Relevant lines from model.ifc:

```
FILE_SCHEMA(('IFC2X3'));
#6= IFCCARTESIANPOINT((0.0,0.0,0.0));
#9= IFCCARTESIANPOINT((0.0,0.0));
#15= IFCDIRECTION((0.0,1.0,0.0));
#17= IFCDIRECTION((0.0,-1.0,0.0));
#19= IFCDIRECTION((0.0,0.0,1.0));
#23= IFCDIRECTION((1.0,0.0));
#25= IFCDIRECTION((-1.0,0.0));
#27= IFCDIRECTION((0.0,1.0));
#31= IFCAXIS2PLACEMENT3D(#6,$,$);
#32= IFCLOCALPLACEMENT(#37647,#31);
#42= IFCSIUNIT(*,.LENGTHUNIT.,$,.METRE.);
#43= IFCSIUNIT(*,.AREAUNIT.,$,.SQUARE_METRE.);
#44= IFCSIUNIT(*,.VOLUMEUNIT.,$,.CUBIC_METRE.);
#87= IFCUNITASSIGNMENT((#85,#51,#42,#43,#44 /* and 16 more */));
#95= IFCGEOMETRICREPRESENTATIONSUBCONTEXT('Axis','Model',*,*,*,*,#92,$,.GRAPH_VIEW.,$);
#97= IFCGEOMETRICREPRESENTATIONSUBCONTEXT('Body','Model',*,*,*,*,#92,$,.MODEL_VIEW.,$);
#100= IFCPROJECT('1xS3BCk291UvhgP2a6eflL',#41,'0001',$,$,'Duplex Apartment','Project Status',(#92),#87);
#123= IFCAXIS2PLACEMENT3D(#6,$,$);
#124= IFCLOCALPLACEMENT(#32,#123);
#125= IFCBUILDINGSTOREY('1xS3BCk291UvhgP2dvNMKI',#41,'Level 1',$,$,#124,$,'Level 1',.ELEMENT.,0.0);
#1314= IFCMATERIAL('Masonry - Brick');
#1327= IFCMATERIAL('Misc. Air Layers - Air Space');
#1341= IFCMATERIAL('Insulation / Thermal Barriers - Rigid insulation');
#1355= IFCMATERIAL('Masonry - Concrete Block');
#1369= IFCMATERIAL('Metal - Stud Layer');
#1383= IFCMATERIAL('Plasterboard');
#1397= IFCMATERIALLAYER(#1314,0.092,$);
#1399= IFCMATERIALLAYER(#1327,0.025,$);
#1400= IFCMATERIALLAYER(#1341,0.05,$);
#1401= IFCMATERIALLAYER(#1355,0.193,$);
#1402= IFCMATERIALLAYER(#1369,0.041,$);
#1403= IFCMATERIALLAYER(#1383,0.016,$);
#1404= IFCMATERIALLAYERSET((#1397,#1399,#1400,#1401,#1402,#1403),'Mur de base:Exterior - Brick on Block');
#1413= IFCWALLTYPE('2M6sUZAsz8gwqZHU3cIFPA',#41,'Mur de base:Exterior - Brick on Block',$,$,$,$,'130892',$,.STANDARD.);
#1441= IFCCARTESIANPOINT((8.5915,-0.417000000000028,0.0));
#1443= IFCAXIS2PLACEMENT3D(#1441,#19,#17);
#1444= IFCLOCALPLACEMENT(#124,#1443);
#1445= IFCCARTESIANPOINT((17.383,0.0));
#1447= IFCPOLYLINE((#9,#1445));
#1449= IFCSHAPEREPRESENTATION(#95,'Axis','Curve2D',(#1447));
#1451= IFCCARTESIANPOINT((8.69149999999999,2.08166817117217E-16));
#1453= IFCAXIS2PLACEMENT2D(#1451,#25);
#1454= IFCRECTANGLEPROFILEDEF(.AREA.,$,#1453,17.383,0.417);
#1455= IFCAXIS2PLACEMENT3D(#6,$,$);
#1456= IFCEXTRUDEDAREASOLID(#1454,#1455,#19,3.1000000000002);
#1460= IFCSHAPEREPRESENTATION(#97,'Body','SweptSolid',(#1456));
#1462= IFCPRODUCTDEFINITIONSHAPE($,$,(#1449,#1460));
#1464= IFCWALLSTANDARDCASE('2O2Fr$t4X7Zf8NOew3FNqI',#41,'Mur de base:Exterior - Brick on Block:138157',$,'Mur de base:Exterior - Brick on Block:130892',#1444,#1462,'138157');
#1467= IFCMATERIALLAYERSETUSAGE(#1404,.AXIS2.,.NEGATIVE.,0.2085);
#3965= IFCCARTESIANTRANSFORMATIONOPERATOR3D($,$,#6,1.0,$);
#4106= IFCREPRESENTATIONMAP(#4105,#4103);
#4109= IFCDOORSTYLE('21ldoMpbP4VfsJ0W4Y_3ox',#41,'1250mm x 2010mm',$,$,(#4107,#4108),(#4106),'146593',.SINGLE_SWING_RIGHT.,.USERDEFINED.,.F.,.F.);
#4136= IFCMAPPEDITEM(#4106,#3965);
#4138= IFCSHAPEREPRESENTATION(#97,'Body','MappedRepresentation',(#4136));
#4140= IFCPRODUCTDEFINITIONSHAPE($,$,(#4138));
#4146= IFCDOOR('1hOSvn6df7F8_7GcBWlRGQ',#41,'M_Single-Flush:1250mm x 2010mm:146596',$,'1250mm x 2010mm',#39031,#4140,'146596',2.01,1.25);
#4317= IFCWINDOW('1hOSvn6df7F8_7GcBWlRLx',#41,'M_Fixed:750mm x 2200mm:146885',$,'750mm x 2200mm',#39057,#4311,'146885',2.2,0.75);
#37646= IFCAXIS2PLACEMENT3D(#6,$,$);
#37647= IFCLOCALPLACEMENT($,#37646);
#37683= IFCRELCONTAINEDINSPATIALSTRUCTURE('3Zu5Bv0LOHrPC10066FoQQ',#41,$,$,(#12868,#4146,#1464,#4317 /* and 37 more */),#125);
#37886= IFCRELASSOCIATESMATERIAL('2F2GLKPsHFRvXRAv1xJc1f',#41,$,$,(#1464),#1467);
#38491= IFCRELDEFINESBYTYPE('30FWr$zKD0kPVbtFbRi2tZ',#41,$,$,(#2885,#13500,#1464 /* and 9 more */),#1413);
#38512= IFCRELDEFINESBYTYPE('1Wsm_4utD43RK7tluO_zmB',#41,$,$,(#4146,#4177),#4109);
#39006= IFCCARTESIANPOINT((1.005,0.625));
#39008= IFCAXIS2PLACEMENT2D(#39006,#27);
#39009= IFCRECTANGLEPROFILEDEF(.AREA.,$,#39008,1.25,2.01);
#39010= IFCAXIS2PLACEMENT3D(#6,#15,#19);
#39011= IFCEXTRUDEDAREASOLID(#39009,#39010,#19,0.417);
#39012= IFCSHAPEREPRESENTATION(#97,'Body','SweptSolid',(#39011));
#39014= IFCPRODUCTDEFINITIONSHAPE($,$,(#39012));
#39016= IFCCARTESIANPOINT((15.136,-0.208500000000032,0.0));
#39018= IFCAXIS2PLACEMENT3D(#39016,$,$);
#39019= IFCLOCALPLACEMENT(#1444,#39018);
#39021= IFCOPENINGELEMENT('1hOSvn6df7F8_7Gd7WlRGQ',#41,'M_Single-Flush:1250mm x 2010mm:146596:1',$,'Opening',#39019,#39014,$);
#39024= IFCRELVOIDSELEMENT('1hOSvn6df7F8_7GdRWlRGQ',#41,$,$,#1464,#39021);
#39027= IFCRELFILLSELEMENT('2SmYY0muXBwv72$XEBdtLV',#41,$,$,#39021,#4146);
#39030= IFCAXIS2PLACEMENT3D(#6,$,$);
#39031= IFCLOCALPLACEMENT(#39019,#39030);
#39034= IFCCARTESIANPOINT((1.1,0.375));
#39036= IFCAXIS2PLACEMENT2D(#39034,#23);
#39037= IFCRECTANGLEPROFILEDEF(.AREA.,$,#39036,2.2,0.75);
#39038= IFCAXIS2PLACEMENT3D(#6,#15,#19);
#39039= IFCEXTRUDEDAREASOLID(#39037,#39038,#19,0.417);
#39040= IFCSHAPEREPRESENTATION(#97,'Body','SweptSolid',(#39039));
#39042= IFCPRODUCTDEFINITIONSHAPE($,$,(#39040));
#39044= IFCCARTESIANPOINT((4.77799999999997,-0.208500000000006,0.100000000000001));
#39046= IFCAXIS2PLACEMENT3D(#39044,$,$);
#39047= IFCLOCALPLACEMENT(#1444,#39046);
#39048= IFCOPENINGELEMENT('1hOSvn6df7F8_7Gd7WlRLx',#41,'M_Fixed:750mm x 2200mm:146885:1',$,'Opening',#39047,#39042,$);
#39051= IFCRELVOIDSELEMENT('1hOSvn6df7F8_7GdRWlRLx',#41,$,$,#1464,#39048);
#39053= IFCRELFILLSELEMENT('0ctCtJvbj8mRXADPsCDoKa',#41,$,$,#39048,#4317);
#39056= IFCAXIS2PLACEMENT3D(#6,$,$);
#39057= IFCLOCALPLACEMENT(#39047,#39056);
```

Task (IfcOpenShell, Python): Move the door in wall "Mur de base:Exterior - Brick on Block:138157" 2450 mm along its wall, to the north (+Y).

```python
import ifcopenshell
import ifcopenshell.api.geometry
import ifcopenshell.util.placement

model = ifcopenshell.open("model.ifc")

door = model.by_guid("1hOSvn6df7F8_7GcBWlRGQ")
opening = door.FillsVoids[0].RelatingOpeningElement
wall = opening.VoidsElements[0].RelatingBuildingElement

wall_matrix = ifcopenshell.util.placement.get_local_placement(wall.ObjectPlacement)
shift = wall_matrix[:3, 0] * -2.45
before = ifcopenshell.util.placement.get_local_placement(door.ObjectPlacement)[:3, 3].copy()

# The door is placed relative to its opening, so it follows when the opening moves.
matrix = ifcopenshell.util.placement.get_local_placement(opening.ObjectPlacement)
matrix[:3, 3] += shift
ifcopenshell.api.geometry.edit_object_placement(
    model, product=opening, matrix=matrix, is_si=False, should_transform_children=True
)

after = ifcopenshell.util.placement.get_local_placement(door.ObjectPlacement)[:3, 3]
print("door moved by", (after - before).round(3) + 0.0)

model.write("model-out.ifc")
```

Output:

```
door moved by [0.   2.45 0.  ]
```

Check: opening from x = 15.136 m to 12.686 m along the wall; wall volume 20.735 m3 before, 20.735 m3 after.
